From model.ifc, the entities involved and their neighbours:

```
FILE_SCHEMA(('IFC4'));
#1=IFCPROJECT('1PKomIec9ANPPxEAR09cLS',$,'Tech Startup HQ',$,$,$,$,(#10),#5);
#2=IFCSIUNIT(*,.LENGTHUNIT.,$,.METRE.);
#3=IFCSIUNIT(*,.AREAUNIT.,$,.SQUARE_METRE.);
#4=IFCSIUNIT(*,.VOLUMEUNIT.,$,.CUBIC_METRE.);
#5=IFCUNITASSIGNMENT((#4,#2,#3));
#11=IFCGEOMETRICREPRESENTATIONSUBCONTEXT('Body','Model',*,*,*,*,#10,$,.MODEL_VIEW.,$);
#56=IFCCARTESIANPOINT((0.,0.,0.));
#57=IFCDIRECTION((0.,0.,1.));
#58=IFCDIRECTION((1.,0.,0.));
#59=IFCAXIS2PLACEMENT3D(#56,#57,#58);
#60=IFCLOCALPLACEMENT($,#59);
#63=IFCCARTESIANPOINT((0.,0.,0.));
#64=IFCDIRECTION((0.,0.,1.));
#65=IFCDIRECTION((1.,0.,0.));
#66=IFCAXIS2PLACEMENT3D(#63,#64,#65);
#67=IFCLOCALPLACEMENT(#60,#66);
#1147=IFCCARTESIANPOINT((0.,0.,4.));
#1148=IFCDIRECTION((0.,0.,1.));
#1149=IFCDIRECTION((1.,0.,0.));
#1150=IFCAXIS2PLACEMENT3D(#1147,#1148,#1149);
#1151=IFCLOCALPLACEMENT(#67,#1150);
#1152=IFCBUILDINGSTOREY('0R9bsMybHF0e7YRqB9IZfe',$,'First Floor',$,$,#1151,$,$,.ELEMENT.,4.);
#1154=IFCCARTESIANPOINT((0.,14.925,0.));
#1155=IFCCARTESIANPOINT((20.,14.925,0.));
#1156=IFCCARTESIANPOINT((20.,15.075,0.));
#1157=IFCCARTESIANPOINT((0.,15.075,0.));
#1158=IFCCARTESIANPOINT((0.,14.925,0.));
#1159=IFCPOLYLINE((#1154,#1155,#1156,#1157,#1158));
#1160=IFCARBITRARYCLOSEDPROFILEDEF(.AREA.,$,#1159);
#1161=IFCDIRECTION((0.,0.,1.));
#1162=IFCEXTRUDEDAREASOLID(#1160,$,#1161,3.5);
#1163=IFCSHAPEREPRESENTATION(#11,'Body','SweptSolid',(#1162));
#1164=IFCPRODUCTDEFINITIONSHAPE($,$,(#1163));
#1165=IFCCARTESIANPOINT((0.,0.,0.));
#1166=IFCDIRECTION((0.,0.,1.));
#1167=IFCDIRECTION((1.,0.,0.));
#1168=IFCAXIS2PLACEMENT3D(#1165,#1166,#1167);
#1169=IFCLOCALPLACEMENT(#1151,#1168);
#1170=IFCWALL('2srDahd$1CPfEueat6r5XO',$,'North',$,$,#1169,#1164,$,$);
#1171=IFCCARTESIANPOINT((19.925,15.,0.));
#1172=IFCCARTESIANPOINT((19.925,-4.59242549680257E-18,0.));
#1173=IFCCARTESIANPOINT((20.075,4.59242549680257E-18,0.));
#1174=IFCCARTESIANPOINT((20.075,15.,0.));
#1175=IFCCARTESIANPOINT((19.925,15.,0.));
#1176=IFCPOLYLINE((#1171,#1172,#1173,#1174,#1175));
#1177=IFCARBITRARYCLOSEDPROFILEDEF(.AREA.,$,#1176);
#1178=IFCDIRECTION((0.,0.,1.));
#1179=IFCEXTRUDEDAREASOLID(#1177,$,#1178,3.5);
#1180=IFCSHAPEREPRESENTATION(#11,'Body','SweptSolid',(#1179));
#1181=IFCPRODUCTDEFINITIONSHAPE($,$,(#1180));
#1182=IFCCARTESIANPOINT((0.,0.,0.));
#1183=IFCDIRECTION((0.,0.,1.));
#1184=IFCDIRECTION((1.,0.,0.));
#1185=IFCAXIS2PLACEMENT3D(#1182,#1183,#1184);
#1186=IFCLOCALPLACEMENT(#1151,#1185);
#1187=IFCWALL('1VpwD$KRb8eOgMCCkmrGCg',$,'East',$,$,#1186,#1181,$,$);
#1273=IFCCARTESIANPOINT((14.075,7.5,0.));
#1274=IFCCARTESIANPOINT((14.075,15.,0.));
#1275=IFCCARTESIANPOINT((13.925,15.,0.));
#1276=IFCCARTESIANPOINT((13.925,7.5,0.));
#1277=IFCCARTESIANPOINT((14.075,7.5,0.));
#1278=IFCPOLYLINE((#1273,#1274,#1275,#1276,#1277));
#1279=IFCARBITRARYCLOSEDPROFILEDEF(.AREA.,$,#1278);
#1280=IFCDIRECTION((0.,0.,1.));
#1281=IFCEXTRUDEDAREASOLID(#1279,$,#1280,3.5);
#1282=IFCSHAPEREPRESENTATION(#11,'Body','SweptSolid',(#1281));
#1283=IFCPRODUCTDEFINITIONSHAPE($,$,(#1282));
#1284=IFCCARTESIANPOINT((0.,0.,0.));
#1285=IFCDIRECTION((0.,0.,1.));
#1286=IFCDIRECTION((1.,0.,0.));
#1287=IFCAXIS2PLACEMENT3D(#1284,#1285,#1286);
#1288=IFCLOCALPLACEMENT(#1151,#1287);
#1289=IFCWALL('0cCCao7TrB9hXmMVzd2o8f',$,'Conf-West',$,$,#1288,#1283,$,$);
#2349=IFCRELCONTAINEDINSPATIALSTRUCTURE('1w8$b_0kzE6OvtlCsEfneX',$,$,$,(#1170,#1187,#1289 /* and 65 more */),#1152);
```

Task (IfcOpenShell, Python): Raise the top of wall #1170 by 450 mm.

```python
import ifcopenshell
import ifcopenshell.geom
import ifcopenshell.util.representation
import ifcopenshell.util.shape
import ifcopenshell.util.unit

model = ifcopenshell.open("model.ifc")
unit_scale = ifcopenshell.util.unit.calculate_unit_scale(model)
settings = ifcopenshell.geom.settings()


def volume(element):
    """Net volume in cubic metres, openings subtracted."""
    shape = ifcopenshell.geom.create_shape(settings, element)
    return ifcopenshell.util.shape.get_volume(shape.geometry)


wall = model.by_guid("2srDahd$1CPfEueat6r5XO")
before = volume(wall)

body = ifcopenshell.util.representation.get_representation(wall, "Model", "Body")
solid = body.Items[0]
old_height = solid.Depth
solid.Depth += 0.45 / unit_scale
after = volume(wall)

print(f"height {old_height:g} -> {solid.Depth:g}, volume {before:.3f} -> {after:.3f} m3")

model.write("model-out.ifc")
```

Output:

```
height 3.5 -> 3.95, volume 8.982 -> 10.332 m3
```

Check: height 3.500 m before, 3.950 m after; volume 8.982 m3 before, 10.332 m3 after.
